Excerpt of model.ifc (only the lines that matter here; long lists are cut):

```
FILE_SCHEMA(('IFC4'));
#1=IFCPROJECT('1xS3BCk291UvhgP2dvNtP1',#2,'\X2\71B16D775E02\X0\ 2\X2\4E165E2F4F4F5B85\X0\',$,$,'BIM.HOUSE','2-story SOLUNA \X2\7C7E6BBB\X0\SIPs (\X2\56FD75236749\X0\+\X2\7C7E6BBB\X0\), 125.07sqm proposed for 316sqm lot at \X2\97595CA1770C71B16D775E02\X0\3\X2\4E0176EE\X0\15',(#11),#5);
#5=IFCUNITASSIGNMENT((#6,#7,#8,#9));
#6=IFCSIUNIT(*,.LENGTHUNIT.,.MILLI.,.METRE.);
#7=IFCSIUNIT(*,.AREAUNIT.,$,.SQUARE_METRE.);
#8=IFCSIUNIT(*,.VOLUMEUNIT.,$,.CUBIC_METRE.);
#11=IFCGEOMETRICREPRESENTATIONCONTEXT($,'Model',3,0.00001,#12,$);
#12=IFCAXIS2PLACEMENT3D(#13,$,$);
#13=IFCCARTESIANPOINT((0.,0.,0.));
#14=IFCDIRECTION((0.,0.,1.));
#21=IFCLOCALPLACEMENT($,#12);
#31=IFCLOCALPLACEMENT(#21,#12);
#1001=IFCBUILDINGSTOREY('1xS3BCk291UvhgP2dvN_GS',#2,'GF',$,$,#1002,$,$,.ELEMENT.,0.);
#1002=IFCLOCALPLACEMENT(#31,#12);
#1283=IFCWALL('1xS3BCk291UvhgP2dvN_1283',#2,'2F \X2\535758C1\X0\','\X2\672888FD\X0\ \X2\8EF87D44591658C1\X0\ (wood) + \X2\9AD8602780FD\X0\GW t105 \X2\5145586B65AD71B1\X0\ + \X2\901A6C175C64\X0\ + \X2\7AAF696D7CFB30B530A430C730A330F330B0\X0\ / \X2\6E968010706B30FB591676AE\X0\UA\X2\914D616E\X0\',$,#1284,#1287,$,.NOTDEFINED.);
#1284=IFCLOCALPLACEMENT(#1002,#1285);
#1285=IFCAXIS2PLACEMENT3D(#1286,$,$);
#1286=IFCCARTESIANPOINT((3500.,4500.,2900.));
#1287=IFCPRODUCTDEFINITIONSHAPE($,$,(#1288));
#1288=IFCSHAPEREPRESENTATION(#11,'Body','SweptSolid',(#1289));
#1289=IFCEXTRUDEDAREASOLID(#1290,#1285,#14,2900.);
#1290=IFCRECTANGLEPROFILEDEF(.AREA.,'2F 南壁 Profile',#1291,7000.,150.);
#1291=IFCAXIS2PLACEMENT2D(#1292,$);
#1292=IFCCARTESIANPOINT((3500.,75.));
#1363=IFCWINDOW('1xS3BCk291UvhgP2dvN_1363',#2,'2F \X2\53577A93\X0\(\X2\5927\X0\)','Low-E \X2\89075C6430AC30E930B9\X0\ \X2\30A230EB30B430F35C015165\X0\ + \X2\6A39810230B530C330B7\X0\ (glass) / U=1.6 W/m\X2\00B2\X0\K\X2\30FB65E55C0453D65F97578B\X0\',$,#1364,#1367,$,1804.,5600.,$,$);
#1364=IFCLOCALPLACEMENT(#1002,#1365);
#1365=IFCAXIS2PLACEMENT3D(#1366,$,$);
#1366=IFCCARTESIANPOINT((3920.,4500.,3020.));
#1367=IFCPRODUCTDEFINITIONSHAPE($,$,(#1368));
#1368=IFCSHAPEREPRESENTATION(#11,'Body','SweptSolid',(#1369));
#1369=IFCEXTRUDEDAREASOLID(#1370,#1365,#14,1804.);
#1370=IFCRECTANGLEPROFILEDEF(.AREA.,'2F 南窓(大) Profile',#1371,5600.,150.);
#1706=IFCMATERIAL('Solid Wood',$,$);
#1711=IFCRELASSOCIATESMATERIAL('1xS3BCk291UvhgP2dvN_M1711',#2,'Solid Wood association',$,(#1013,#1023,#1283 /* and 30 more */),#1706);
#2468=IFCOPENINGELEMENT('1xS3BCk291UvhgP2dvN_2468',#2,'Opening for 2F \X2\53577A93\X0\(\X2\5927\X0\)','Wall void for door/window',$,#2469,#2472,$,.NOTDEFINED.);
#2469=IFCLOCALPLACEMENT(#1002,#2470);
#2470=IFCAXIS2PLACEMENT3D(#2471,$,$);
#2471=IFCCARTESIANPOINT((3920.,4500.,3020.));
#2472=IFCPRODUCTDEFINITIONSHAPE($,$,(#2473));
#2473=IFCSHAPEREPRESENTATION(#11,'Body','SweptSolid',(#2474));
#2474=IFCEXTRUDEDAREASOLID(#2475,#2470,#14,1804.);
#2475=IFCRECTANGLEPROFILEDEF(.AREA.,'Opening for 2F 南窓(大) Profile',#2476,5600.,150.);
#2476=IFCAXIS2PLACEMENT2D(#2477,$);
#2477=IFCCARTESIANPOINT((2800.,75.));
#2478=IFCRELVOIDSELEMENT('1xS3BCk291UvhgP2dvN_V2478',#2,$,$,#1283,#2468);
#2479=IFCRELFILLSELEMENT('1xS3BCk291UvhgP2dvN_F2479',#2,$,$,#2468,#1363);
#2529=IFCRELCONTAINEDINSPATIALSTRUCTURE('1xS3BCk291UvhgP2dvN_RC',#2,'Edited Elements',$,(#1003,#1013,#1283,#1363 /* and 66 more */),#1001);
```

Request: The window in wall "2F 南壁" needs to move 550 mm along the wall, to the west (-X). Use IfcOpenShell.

```python
import ifcopenshell
import ifcopenshell.api.geometry
import ifcopenshell.util.placement

model = ifcopenshell.open("model.ifc")

window = model.by_guid("1xS3BCk291UvhgP2dvN_1363")
opening = window.FillsVoids[0].RelatingOpeningElement
wall = opening.VoidsElements[0].RelatingBuildingElement

wall_matrix = ifcopenshell.util.placement.get_local_placement(wall.ObjectPlacement)
shift = wall_matrix[:3, 0] * -550.0
before = ifcopenshell.util.placement.get_local_placement(window.ObjectPlacement)[:3, 3].copy()

# The window is not placed relative to its opening, so move both.
for product in (opening, window):
    matrix = ifcopenshell.util.placement.get_local_placement(product.ObjectPlacement)
    matrix[:3, 3] += shift
    ifcopenshell.api.geometry.edit_object_placement(model, product=product, matrix=matrix, is_si=False)

after = ifcopenshell.util.placement.get_local_placement(window.ObjectPlacement)[:3, 3]
print("window moved by", (after - before).round(3) + 0.0)

model.write("model_edited.ifc")
```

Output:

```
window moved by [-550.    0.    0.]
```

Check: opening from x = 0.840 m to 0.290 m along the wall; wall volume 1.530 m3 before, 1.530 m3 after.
